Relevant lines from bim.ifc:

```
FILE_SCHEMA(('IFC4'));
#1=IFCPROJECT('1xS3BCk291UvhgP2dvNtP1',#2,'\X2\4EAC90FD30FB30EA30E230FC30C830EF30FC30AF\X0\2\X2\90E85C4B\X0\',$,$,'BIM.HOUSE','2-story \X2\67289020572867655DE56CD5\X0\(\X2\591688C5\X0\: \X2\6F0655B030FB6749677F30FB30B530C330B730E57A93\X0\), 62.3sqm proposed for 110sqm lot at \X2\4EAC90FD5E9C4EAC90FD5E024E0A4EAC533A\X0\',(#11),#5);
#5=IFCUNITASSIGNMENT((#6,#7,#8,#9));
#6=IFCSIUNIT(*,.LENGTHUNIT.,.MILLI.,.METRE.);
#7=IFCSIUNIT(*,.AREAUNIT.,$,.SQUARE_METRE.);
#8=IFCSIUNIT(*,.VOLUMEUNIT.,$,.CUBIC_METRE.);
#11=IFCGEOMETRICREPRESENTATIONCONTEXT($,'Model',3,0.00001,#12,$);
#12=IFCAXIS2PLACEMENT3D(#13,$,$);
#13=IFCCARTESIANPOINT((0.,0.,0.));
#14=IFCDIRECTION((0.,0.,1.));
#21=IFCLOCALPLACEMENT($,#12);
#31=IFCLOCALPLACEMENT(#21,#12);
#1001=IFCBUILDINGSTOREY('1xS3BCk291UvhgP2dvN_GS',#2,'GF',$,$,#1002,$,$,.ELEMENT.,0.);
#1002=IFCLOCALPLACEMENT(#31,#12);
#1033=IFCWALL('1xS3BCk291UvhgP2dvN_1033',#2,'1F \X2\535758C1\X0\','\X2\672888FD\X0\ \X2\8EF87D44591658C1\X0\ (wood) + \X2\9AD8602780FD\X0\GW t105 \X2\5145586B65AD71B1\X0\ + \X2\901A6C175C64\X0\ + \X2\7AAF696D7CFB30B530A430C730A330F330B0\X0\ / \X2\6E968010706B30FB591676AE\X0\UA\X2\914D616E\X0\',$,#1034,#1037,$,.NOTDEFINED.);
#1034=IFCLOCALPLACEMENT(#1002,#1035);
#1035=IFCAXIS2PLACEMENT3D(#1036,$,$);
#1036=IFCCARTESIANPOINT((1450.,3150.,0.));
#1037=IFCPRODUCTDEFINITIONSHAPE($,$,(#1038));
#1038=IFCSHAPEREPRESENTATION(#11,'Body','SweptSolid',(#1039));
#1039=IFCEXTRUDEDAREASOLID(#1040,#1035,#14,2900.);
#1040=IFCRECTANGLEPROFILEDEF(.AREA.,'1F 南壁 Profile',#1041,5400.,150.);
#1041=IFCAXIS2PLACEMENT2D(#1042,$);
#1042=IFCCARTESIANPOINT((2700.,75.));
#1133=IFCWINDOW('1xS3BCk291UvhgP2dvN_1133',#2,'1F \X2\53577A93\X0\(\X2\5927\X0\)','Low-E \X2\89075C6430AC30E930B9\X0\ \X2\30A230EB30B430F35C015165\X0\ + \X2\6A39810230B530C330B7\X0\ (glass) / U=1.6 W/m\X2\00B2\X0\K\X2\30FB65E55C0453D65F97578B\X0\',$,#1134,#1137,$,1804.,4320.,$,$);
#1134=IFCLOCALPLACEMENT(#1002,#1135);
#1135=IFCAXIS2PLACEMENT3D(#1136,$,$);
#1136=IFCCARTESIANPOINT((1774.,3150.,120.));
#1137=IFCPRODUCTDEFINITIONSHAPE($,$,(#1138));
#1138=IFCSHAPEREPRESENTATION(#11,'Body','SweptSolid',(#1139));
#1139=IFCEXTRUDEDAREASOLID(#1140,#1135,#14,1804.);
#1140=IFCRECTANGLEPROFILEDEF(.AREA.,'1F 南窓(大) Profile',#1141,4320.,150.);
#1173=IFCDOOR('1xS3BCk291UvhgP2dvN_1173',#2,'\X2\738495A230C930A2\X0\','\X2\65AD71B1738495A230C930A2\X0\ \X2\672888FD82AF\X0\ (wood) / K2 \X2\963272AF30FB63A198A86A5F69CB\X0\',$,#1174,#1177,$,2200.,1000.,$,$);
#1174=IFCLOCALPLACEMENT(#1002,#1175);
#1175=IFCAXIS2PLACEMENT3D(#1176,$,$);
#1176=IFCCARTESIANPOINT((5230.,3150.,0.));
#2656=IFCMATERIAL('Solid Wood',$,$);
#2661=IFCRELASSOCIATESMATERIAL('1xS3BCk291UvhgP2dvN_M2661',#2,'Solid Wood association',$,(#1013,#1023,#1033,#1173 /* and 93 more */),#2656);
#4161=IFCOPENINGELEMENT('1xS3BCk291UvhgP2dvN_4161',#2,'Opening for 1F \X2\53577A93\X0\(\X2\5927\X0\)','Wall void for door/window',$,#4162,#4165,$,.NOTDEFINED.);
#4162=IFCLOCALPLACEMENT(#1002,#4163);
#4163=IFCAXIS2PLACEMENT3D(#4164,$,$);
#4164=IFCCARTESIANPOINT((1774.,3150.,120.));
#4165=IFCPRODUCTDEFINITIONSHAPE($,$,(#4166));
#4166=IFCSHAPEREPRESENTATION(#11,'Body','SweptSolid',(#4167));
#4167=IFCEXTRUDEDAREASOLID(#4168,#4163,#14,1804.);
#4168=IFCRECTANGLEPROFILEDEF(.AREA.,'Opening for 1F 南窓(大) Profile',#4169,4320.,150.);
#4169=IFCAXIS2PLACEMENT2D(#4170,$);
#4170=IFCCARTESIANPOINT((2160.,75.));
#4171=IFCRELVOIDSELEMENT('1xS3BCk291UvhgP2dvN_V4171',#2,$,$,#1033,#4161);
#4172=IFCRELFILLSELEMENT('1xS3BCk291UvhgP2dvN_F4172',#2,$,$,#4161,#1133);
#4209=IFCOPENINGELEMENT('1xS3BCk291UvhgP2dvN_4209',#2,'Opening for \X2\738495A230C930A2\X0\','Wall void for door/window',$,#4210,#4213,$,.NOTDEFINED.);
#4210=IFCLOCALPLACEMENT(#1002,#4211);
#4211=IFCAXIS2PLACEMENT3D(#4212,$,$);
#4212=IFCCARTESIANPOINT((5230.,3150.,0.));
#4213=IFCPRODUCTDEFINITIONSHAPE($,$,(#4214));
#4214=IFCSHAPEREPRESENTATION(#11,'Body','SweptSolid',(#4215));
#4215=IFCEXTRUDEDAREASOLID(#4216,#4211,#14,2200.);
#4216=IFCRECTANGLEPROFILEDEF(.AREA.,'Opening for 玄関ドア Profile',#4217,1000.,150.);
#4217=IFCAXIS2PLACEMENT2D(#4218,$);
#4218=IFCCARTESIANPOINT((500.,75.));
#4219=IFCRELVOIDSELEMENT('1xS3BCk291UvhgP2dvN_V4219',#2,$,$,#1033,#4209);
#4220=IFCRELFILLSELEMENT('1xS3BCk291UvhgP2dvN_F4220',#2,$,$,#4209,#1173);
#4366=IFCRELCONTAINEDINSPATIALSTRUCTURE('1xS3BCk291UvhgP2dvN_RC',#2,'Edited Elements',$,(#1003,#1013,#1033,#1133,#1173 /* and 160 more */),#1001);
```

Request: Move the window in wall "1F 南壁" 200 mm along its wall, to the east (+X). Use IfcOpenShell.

```python
import ifcopenshell
import ifcopenshell.api.geometry
import ifcopenshell.util.placement

model = ifcopenshell.open("bim.ifc")

window = model.by_id(1133)
opening = window.FillsVoids[0].RelatingOpeningElement
wall = opening.VoidsElements[0].RelatingBuildingElement

wall_matrix = ifcopenshell.util.placement.get_local_placement(wall.ObjectPlacement)
shift = wall_matrix[:3, 0] * 200.0
before = ifcopenshell.util.placement.get_local_placement(window.ObjectPlacement)[:3, 3].copy()

# The window is not placed relative to its opening, so move both.
for product in (opening, window):
    matrix = ifcopenshell.util.placement.get_local_placement(product.ObjectPlacement)
    matrix[:3, 3] += shift
    ifcopenshell.api.geometry.edit_object_placement(model, product=product, matrix=matrix, is_si=False)

after = ifcopenshell.util.placement.get_local_placement(window.ObjectPlacement)[:3, 3]
print("window moved by", (after - before).round(3) + 0.0)

model.write("bim_edited.ifc")
```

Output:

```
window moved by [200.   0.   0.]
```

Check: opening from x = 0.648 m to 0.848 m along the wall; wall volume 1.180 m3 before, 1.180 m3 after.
